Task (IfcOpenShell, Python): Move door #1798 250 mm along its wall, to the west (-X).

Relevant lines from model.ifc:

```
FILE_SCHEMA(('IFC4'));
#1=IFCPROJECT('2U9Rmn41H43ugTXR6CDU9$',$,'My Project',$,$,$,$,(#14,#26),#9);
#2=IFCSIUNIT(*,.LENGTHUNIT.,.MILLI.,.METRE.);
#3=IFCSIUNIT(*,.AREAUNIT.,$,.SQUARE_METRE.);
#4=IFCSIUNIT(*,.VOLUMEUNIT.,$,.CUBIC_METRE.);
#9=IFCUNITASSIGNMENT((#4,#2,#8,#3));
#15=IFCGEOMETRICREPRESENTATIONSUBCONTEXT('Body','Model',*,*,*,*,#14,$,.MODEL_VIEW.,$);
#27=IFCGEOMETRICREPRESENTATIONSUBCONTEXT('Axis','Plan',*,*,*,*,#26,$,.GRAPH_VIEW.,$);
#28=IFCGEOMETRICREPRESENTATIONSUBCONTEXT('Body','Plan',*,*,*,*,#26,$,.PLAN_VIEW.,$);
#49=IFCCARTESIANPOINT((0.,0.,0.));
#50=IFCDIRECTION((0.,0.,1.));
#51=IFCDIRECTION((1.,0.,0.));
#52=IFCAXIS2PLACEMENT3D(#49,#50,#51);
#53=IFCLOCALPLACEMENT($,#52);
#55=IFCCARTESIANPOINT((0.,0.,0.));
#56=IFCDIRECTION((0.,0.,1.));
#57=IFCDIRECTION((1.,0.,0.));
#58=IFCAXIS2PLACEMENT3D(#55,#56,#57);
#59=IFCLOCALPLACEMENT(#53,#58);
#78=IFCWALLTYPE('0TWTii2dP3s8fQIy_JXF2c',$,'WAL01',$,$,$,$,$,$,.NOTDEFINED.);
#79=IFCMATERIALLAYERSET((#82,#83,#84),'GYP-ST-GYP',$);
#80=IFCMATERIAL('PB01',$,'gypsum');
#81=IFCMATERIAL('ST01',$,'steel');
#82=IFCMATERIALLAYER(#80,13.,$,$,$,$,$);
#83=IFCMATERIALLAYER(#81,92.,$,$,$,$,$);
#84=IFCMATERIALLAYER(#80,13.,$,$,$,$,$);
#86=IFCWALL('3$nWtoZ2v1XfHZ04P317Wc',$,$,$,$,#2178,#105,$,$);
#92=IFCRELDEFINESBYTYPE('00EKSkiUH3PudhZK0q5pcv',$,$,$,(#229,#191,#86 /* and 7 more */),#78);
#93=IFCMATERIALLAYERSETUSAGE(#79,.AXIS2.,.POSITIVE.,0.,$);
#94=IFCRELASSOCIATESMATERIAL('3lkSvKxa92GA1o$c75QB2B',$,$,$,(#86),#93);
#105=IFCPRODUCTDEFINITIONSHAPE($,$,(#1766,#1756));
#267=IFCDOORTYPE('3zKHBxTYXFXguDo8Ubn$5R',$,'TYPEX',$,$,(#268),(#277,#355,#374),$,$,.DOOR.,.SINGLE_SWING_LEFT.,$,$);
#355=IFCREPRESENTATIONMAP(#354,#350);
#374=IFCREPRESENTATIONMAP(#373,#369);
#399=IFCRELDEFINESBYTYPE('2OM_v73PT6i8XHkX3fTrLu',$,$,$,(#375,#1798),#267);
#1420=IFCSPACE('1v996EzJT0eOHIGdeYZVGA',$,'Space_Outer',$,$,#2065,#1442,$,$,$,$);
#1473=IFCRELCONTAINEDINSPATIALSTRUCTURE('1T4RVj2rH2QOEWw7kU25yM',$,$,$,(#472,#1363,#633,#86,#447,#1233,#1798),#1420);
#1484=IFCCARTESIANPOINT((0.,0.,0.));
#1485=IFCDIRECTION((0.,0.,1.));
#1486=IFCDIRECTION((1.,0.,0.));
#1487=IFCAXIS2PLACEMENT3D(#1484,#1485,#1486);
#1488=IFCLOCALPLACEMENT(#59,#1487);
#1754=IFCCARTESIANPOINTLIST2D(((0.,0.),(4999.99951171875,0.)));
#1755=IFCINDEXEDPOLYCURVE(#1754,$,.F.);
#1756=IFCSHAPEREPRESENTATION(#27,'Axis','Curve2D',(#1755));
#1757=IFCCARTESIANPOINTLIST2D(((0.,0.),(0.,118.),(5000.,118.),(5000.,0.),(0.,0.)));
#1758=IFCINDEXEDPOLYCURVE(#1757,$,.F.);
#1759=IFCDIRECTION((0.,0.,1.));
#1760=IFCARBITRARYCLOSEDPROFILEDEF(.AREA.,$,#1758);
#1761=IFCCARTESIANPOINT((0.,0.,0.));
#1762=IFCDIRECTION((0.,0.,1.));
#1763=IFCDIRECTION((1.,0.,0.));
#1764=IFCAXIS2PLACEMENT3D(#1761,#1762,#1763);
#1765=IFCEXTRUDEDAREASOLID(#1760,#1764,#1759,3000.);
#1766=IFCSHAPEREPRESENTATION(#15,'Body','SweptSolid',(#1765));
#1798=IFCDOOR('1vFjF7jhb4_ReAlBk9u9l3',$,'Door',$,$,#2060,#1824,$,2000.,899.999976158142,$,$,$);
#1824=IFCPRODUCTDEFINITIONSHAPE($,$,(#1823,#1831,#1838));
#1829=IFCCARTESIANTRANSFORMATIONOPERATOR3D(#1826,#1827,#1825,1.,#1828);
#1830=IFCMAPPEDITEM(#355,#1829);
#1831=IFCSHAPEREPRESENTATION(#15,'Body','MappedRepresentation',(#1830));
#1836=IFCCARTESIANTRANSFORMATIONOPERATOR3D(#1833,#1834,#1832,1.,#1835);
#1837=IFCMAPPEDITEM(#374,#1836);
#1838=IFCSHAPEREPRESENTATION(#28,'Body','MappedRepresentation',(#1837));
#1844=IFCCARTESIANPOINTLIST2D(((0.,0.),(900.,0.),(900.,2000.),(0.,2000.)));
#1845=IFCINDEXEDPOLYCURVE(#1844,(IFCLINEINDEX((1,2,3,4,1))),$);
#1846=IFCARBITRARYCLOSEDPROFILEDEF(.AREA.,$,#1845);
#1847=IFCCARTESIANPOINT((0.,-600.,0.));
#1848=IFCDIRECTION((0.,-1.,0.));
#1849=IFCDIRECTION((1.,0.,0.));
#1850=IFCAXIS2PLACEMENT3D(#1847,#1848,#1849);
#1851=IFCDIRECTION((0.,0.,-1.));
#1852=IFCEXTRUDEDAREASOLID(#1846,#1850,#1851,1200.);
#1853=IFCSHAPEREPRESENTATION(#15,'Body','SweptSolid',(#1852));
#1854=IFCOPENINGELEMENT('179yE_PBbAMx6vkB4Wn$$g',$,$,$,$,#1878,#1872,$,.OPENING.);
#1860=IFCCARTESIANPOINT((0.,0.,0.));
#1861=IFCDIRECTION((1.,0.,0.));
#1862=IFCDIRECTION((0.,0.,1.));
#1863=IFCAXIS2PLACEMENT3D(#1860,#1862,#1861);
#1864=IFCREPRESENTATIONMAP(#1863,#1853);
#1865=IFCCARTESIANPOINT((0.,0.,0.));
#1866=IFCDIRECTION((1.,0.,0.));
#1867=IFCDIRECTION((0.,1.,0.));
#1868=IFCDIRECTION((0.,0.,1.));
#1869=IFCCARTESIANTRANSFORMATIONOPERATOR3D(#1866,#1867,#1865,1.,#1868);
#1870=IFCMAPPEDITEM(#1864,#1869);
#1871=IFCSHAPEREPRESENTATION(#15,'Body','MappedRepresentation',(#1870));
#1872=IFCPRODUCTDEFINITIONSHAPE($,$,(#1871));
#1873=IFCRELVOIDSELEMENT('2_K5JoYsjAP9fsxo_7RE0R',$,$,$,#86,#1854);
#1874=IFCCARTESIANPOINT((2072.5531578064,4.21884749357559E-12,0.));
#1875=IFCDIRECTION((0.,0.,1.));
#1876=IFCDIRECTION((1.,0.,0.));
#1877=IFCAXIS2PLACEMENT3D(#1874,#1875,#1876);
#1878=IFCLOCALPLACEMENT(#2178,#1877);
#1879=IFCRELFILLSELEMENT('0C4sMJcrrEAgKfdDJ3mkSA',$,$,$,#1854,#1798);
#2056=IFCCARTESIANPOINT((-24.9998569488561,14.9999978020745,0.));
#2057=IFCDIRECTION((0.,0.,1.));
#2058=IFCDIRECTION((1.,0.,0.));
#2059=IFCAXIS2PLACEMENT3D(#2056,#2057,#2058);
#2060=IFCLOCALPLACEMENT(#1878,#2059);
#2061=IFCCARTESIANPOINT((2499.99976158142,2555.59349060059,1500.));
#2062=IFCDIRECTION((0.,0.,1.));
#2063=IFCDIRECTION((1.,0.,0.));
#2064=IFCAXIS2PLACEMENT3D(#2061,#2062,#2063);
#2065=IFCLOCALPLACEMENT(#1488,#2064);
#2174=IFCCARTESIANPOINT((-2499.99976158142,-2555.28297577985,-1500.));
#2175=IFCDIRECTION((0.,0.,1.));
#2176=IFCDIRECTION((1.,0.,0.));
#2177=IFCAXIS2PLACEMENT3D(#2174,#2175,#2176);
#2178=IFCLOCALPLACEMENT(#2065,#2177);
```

```python
import ifcopenshell
import ifcopenshell.api.geometry
import ifcopenshell.util.placement
import ifcopenshell.util.unit

model = ifcopenshell.open("model.ifc")
unit_scale = ifcopenshell.util.unit.calculate_unit_scale(model)

door = model.by_id(1798)
opening = door.FillsVoids[0].RelatingOpeningElement
wall = opening.VoidsElements[0].RelatingBuildingElement

wall_matrix = ifcopenshell.util.placement.get_local_placement(wall.ObjectPlacement)
shift = wall_matrix[:3, 0] * -0.25 / unit_scale
before = ifcopenshell.util.placement.get_local_placement(door.ObjectPlacement)[:3, 3].copy()

# The door is placed relative to its opening, so it follows when the opening moves.
matrix = ifcopenshell.util.placement.get_local_placement(opening.ObjectPlacement)
matrix[:3, 3] += shift
ifcopenshell.api.geometry.edit_object_placement(
    model, product=opening, matrix=matrix, is_si=False, should_transform_children=True
)

after = ifcopenshell.util.placement.get_local_placement(door.ObjectPlacement)[:3, 3]
print("door moved by", (after - before).round(3) + 0.0)

model.write("model_updated.ifc")
```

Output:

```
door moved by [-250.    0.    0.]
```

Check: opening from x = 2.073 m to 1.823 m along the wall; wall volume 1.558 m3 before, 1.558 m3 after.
